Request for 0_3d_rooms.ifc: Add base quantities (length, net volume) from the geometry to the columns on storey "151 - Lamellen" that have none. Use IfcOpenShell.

First a look at what the model holds.

```python
import ifcopenshell
import ifcopenshell.util.element
import ifcopenshell.util.unit

model = ifcopenshell.open("0_3d_rooms.ifc")
print(model.schema)
for unit_type in ("LENGTHUNIT", "AREAUNIT", "VOLUMEUNIT"):
    print(unit_type, ifcopenshell.util.unit.calculate_unit_scale(model, unit_type))
storey = next(s for s in model.by_type("IfcBuildingStorey") if s.Name == "151 - Lamellen")
columns = [e for e in ifcopenshell.util.element.get_decomposition(storey) if e.is_a("IfcColumn")]
for e in sorted(columns, key=lambda e: e.id()):
    print(e.id(), e.is_a(), e.Name, list(ifcopenshell.util.element.get_psets(e, qtos_only=True)), sep=" | ")
```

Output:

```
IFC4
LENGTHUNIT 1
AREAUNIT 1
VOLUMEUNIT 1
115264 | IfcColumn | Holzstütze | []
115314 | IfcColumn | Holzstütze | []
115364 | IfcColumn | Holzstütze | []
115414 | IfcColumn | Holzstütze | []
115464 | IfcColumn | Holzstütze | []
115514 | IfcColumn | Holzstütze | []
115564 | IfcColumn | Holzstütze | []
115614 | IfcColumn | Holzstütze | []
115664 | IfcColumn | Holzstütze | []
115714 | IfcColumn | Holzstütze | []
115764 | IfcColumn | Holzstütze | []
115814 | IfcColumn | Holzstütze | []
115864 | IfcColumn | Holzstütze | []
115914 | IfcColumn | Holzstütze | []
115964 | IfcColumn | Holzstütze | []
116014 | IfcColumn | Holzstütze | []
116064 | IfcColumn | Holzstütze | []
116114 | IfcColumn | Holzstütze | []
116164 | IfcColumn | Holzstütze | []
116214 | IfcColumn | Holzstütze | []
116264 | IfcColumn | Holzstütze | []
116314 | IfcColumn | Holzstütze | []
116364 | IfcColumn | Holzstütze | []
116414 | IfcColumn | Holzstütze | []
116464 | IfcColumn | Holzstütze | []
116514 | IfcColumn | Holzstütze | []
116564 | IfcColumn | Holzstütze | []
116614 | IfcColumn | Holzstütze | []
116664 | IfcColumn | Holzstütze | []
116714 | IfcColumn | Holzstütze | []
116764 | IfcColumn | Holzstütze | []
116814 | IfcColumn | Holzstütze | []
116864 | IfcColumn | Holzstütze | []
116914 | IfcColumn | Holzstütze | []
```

```python
import ifcopenshell
import ifcopenshell.api.pset
import ifcopenshell.geom
import ifcopenshell.util.element
import ifcopenshell.util.shape
import ifcopenshell.util.unit

model = ifcopenshell.open("0_3d_rooms.ifc")
unit_scale = ifcopenshell.util.unit.calculate_unit_scale(model)
volume_scale = ifcopenshell.util.unit.calculate_unit_scale(model, "VOLUMEUNIT")
settings = ifcopenshell.geom.settings()

storey = next(s for s in model.by_type("IfcBuildingStorey") if s.Name == "151 - Lamellen")
columns = [e for e in ifcopenshell.util.element.get_decomposition(storey) if e.is_a("IfcColumn")]

for e in sorted(columns, key=lambda e: e.id()):
    if ifcopenshell.util.element.get_psets(e, qtos_only=True, should_inherit=False):
        continue
    # Geometry comes back in metres, in the element's own axes.
    shape = ifcopenshell.geom.create_shape(settings, e)
    values = {
        "Length": ifcopenshell.util.shape.get_z(shape.geometry) / unit_scale,
        "NetVolume": ifcopenshell.util.shape.get_volume(shape.geometry) / volume_scale,
    }
    qto = ifcopenshell.api.pset.add_qto(model, product=e, name="Qto_ColumnBaseQuantities")
    ifcopenshell.api.pset.edit_qto(model, qto=qto, properties=values)
    print(e.id(), {k: round(v, 3) for k, v in values.items()})

model.write("0_3d_rooms-out.ifc")
```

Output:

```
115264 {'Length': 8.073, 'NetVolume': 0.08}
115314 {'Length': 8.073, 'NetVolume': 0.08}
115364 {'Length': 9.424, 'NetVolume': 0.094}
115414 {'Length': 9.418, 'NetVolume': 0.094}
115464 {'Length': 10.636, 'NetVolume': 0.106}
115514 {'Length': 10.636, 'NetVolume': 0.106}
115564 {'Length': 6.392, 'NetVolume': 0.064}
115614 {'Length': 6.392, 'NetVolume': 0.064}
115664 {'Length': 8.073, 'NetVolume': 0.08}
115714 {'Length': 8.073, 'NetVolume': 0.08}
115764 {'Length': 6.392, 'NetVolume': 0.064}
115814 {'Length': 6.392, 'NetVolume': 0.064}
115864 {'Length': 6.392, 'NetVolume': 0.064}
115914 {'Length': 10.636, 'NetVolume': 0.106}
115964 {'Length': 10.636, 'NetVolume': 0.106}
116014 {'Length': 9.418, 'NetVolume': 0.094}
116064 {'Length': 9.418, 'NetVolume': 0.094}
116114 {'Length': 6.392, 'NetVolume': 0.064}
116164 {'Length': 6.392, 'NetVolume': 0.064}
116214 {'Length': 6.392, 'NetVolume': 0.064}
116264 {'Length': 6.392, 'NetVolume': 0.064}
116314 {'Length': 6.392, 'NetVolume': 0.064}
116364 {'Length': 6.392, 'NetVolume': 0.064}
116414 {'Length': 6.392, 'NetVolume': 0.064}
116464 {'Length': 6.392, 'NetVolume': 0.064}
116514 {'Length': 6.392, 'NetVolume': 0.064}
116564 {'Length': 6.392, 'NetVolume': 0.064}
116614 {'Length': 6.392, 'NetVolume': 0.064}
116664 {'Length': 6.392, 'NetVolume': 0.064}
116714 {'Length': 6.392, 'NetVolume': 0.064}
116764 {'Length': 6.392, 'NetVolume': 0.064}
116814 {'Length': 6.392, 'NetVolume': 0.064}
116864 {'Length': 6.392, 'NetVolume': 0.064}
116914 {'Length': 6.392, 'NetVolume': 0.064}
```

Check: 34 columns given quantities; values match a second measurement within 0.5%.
